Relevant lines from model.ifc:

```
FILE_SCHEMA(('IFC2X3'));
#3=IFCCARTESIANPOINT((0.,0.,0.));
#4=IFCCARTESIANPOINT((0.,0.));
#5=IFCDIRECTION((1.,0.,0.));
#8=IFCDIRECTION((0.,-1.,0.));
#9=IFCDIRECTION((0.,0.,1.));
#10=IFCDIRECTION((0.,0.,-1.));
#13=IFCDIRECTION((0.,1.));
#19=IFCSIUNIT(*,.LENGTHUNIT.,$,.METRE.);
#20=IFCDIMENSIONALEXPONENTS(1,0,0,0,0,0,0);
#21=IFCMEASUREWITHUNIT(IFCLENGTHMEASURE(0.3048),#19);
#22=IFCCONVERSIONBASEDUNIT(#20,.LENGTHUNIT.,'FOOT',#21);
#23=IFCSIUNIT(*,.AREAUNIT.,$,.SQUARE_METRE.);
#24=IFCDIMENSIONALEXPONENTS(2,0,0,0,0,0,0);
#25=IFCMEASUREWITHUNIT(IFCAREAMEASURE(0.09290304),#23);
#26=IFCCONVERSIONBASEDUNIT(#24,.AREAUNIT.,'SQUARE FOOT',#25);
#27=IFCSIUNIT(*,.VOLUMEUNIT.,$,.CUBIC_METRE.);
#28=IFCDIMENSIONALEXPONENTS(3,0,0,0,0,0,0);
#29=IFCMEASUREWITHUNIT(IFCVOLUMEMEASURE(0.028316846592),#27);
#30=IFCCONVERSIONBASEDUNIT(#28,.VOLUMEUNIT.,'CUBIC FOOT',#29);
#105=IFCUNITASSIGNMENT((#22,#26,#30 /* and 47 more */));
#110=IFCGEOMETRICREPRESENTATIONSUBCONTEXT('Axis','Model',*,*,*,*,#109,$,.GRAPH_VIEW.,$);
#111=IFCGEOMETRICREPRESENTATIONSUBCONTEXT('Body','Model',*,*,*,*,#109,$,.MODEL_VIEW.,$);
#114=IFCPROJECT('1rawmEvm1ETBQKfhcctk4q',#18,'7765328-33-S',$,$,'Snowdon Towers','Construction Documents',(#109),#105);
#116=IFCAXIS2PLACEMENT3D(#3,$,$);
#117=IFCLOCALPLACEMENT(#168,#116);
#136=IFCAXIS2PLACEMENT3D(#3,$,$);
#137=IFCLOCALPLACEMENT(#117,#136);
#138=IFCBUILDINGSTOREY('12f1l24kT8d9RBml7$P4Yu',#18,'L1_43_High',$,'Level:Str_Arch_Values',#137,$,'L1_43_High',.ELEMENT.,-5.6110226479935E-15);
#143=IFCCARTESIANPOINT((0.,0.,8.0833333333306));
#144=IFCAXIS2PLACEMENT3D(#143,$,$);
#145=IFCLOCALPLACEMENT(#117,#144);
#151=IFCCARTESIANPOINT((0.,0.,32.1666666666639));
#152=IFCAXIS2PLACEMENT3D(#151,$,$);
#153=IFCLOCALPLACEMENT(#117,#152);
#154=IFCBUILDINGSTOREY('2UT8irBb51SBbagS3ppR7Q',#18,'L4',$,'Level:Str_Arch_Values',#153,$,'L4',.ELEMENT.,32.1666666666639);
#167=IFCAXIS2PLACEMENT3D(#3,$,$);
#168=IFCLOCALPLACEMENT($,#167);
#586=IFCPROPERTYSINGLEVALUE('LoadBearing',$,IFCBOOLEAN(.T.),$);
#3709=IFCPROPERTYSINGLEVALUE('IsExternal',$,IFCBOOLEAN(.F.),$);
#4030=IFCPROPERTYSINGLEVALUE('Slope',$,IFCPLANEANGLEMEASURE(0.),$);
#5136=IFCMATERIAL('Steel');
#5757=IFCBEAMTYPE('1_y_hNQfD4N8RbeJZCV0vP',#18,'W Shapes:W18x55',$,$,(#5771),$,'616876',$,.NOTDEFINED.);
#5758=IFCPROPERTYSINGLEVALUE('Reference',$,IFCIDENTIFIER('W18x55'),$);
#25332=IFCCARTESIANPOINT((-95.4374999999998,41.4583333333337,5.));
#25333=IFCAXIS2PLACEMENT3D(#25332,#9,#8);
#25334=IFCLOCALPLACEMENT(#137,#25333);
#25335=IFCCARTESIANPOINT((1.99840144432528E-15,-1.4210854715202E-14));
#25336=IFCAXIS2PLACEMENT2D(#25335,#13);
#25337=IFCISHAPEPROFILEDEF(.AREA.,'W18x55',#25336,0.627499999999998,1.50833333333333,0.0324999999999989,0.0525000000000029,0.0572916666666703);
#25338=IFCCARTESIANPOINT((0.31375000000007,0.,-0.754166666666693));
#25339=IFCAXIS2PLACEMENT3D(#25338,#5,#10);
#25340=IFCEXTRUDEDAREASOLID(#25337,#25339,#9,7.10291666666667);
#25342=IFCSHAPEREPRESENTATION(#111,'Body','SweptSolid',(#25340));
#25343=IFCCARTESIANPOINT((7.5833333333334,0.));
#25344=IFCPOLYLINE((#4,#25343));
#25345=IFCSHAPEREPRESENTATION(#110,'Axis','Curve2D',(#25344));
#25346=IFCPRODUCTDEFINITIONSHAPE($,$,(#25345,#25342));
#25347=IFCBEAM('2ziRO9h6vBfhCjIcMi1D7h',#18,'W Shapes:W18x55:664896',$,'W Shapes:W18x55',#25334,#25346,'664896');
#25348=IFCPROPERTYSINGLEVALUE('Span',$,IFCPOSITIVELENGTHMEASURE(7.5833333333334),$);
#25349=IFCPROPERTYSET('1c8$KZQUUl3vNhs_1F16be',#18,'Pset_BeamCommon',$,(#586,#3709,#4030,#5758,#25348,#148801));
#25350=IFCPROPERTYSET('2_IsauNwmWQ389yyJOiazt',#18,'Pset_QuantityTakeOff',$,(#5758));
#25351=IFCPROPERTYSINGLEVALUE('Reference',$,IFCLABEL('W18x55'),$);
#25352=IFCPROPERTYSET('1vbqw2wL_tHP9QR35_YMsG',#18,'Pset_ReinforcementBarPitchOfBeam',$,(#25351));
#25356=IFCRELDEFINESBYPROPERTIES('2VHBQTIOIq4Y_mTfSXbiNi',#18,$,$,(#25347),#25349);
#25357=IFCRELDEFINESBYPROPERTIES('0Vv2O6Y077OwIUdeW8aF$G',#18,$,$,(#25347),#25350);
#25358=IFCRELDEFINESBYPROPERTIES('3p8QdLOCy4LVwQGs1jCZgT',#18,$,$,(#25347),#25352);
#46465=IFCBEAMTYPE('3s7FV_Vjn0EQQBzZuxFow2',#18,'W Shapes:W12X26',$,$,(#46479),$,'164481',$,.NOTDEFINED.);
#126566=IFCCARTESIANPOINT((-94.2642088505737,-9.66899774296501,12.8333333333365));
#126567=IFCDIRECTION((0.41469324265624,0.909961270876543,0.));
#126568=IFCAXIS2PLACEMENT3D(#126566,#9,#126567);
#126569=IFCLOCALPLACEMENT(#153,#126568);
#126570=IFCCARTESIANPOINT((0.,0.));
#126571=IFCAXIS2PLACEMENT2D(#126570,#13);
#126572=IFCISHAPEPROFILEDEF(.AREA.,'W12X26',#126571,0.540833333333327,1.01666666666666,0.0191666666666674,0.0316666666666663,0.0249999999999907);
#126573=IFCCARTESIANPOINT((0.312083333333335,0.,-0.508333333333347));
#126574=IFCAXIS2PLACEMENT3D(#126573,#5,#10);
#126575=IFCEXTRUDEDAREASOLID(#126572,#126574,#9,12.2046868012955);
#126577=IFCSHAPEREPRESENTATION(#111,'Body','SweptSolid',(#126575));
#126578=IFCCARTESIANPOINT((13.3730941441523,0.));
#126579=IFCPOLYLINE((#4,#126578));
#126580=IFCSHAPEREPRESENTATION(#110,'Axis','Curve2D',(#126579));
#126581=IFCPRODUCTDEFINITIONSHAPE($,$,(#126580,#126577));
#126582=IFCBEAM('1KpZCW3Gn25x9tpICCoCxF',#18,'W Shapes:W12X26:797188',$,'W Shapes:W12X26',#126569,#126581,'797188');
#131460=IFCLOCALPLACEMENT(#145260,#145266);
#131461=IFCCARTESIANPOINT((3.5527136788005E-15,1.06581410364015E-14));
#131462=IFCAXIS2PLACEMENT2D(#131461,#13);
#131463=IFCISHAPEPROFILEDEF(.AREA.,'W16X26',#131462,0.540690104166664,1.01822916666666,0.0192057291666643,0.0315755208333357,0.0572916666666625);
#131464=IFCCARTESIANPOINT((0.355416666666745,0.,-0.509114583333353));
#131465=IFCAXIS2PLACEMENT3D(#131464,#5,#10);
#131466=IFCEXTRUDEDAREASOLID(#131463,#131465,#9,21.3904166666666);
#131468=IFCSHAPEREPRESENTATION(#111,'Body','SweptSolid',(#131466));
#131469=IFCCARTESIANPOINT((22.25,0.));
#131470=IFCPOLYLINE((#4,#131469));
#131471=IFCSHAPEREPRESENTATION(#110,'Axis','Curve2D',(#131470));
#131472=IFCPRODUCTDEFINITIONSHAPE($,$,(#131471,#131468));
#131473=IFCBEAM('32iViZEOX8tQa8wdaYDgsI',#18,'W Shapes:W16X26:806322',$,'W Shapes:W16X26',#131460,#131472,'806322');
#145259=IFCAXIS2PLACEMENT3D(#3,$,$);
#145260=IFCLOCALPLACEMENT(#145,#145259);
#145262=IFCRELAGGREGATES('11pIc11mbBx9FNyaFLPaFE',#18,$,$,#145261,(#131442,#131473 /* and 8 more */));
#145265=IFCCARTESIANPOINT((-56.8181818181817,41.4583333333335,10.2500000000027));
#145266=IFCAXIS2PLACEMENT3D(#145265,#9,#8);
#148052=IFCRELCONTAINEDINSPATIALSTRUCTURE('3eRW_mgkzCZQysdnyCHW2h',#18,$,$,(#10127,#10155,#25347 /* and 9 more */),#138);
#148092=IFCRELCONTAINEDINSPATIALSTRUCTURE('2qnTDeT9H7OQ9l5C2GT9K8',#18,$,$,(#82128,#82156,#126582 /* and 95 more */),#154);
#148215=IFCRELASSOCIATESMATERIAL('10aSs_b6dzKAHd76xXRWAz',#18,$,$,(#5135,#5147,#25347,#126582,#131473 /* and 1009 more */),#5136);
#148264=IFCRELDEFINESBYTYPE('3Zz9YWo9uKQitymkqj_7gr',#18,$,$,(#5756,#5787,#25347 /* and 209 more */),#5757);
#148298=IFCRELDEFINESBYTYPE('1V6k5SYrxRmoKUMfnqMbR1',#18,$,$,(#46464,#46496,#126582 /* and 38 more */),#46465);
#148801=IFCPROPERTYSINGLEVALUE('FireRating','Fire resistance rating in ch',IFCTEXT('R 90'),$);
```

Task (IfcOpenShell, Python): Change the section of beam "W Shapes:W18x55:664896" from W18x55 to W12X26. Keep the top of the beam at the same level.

```python
import ifcopenshell
import ifcopenshell.api.pset
import ifcopenshell.api.type
import ifcopenshell.util.element
import ifcopenshell.util.representation

model = ifcopenshell.open("model.ifc")

member = model.by_guid("2ziRO9h6vBfhCjIcMi1D7h")
source = next(p for p in model.by_type("IfcIShapeProfileDef") if p.ProfileName == "W12X26")

body = ifcopenshell.util.representation.get_representation(member, "Model", "Body")
solid = body.Items[0]
old_profile = solid.SweptArea

# Copy the section's sizes but keep this member's own profile position.
profile = ifcopenshell.util.element.copy(model, source)
# Profiles are centred, so shift by half the change in depth to hold the top.
shift = (old_profile.OverallDepth - profile.OverallDepth) / 2
x, y = old_profile.Position.Location.Coordinates
up = (-1.0, 0.0)  # upwards, in the solid's own plane
location = model.createIfcCartesianPoint((x + up[0] * shift, y + up[1] * shift))
profile.Position = model.createIfcAxis2Placement2D(location, old_profile.Position.RefDirection)
solid.SweptArea = profile
if not model.get_total_inverses(old_profile):
    ifcopenshell.util.element.remove_deep2(model, old_profile)

new_type = model.by_guid("3s7FV_Vjn0EQQBzZuxFow2")
ifcopenshell.api.type.assign_type(
    model, related_objects=[member], relating_type=new_type, should_map_representations=False
)
member.Name = member.Name.replace("W18x55", "W12X26")
member.ObjectType = "W Shapes:W12X26"
pset = model.by_id(ifcopenshell.util.element.get_pset(member, "Pset_BeamCommon", should_inherit=False)["id"])
ifcopenshell.api.pset.edit_pset(model, pset=pset, properties={"Reference": "W12X26"})
pset = model.by_id(ifcopenshell.util.element.get_pset(member, "Pset_QuantityTakeOff", should_inherit=False)["id"])
ifcopenshell.api.pset.edit_pset(model, pset=pset, properties={"Reference": "W12X26"})
pset = model.by_id(ifcopenshell.util.element.get_pset(member, "Pset_ReinforcementBarPitchOfBeam", should_inherit=False)["id"])
ifcopenshell.api.pset.edit_pset(model, pset=pset, properties={"Reference": "W12X26"})

print(solid.SweptArea)

model.write("model_rev.ifc")
```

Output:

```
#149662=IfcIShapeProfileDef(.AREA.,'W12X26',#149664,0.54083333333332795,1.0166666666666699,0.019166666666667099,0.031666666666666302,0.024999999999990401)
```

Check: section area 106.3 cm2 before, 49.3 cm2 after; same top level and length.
